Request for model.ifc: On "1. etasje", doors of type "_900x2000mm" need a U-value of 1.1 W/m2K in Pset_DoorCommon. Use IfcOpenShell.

First a look at what the model holds.

```python
import ifcopenshell
import ifcopenshell.util.element

model = ifcopenshell.open("model.ifc")
print(model.schema)
storey = next(s for s in model.by_type("IfcBuildingStorey") if s.Name == "1. etasje")
doors = [e for e in ifcopenshell.util.element.get_decomposition(storey) if e.is_a("IfcDoor")]
seen = {}
for e in doors:
    element_type = ifcopenshell.util.element.get_type(e)
    key = (element_type.Name if element_type != e and element_type else None, ifcopenshell.util.element.get_pset(e, "Pset_DoorCommon", "ThermalTransmittance"))
    seen[key] = seen.get(key, 0) + 1
for (name, value), count in sorted(seen.items(), key=str):
    print(count, "x", name, "|", value)
```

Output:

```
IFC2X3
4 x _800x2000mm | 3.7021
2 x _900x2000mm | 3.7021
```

```python
import ifcopenshell
import ifcopenshell.api.pset
import ifcopenshell.util.element

model = ifcopenshell.open("model.ifc")

storey = next(s for s in model.by_type("IfcBuildingStorey") if s.Name == "1. etasje")
doors = [e for e in ifcopenshell.util.element.get_decomposition(storey) if e.is_a("IfcDoor")]

count = 0
for e in doors:
    element_type = ifcopenshell.util.element.get_type(e)
    if element_type in (None, e) or element_type.Name != "_900x2000mm":
        continue
    # add_pset returns the element's existing set when there is one.
    pset = ifcopenshell.api.pset.add_pset(model, product=e, name="Pset_DoorCommon")
    ifcopenshell.api.pset.edit_pset(model, pset=pset, properties={"ThermalTransmittance": 1.1})
    count += 1

print(count, "doors updated")

model.write("model_v2.ifc")
```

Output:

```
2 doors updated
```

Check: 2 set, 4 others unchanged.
